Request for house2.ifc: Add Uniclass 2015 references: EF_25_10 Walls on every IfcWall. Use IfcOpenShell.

First a look at what the model holds.

```python
import ifcopenshell

model = ifcopenshell.open("house2.ifc")
print(model.schema)
print("classifications:", [c.Name for c in model.by_type("IfcClassification")])
for ifc_class in ("IfcDoor", "IfcRoof", "IfcStair", "IfcWall", "IfcWindow"):
    print(ifc_class, len(model.by_type(ifc_class)))
```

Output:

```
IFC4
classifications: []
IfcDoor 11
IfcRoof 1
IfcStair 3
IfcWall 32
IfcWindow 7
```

```python
import ifcopenshell
import ifcopenshell.api.classification

model = ifcopenshell.open("house2.ifc")

system = ifcopenshell.api.classification.add_classification(model, classification="Uniclass 2015")

codes = {
    "IfcWall": ("EF_25_10", "Walls"),
}
for ifc_class, (code, name) in codes.items():
    products = model.by_type(ifc_class)
    ifcopenshell.api.classification.add_reference(
        model, products=products, classification=system, identification=code, name=name
    )
    print(code, len(products))

model.write("house2-out.ifc")
```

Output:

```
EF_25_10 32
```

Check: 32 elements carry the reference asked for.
